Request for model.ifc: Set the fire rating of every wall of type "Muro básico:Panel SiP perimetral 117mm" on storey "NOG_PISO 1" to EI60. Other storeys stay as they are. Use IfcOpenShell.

First a look at what the model holds.

```python
import ifcopenshell
import ifcopenshell.util.element

model = ifcopenshell.open("model.ifc")
print(model.schema)
storey = next(s for s in model.by_type("IfcBuildingStorey") if s.Name == "NOG_PISO 1")
walls = [e for e in ifcopenshell.util.element.get_decomposition(storey) if e.is_a("IfcWall")]
seen = {}
for e in walls:
    element_type = ifcopenshell.util.element.get_type(e)
    key = (element_type.Name if element_type != e and element_type else None, ifcopenshell.util.element.get_pset(e, "Pset_WallCommon", "FireRating"))
    seen[key] = seen.get(key, 0) + 1
for (name, value), count in sorted(seen.items(), key=str):
    print(count, "x", name, "|", value)
```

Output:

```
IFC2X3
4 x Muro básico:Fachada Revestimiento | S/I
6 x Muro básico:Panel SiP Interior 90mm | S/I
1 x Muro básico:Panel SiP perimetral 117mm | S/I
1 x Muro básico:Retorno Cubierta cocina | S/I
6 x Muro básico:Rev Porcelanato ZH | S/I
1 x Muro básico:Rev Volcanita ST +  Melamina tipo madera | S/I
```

```python
import ifcopenshell
import ifcopenshell.api.pset
import ifcopenshell.util.element

model = ifcopenshell.open("model.ifc")

storey = next(s for s in model.by_type("IfcBuildingStorey") if s.Name == "NOG_PISO 1")
walls = [e for e in ifcopenshell.util.element.get_decomposition(storey) if e.is_a("IfcWall")]

count = 0
for e in walls:
    element_type = ifcopenshell.util.element.get_type(e)
    if element_type in (None, e) or element_type.Name != "Muro básico:Panel SiP perimetral 117mm":
        continue
    # add_pset returns the element's existing set when there is one.
    pset = ifcopenshell.api.pset.add_pset(model, product=e, name="Pset_WallCommon")
    ifcopenshell.api.pset.edit_pset(model, pset=pset, properties={"FireRating": "EI60"})
    count += 1

print(count, "walls updated")

model.write("model_updated.ifc")
```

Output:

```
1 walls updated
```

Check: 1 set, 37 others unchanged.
